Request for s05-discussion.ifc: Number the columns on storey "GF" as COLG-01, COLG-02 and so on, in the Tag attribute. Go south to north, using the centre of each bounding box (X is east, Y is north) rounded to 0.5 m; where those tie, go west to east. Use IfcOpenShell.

First a look at what the model holds.

```python
import ifcopenshell
import ifcopenshell.util.element
import ifcopenshell.util.placement

model = ifcopenshell.open("s05-discussion.ifc")
print(model.schema)
storey = next(s for s in model.by_type("IfcBuildingStorey") if s.Name == "GF")
columns = [e for e in ifcopenshell.util.element.get_decomposition(storey) if e.is_a("IfcColumn")]
for e in sorted(columns, key=lambda e: e.id()):
    origin = ifcopenshell.util.placement.get_local_placement(e.ObjectPlacement)[:3, 3]
    print(e.id(), e.Tag, e.Name, origin.round(2) + 0.0, sep=" | ")
```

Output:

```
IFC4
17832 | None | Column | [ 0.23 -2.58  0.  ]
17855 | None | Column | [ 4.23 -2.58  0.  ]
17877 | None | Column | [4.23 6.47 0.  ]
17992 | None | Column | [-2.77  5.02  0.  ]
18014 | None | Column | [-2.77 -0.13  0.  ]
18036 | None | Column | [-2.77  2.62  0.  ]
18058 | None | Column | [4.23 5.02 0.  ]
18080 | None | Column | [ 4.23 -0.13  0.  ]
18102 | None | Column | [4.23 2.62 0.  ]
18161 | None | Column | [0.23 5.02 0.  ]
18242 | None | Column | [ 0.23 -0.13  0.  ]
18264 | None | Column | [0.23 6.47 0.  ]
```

```python
import ifcopenshell
import ifcopenshell.geom
import ifcopenshell.util.element
import ifcopenshell.util.shape

model = ifcopenshell.open("s05-discussion.ifc")
settings = ifcopenshell.geom.settings()
settings.set("use-world-coords", True)


def centre(element):
    shape = ifcopenshell.geom.create_shape(settings, element)
    return ifcopenshell.util.shape.get_bbox_centroid(shape.geometry)


storey = next(s for s in model.by_type("IfcBuildingStorey") if s.Name == "GF")
columns = [e for e in ifcopenshell.util.element.get_decomposition(storey) if e.is_a("IfcColumn")]

# Insertion points can sit at a corner or the storey origin, so sort by the geometry (in metres).
centres = {e: centre(e) for e in columns}
columns.sort(key=lambda e: (round(centres[e][1] / 0.5), centres[e][0]))

for i, e in enumerate(columns, start=1):
    number = f"COLG-{i:02d}"
    e.Tag = number
    print(e.id(), number)

model.write("s05-discussion_updated.ifc")
```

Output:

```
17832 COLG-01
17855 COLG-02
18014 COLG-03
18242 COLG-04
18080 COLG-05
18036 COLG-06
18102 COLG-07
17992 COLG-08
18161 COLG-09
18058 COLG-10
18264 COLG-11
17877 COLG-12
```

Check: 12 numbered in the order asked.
